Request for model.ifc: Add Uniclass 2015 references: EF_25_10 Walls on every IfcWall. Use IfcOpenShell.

First a look at what the model holds.

```python
import ifcopenshell

model = ifcopenshell.open("model.ifc")
print(model.schema)
print("classifications:", [c.Name for c in model.by_type("IfcClassification")])
for ifc_class in ("IfcDoor", "IfcRoof", "IfcStair", "IfcWall", "IfcWindow"):
    print(ifc_class, len(model.by_type(ifc_class)))
```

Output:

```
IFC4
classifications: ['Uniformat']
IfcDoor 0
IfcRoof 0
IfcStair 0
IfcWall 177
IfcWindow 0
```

```python
import ifcopenshell
import ifcopenshell.api.classification

model = ifcopenshell.open("model.ifc")

system = ifcopenshell.api.classification.add_classification(model, classification="Uniclass 2015")

codes = {
    "IfcWall": ("EF_25_10", "Walls"),
}
for ifc_class, (code, name) in codes.items():
    products = model.by_type(ifc_class)
    ifcopenshell.api.classification.add_reference(
        model, products=products, classification=system, identification=code, name=name
    )
    print(code, len(products))

model.write("model_v2.ifc")
```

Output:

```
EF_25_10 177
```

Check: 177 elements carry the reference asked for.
